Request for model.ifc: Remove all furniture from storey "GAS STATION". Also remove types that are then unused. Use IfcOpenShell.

First a look at what the model holds.

```python
import ifcopenshell
import ifcopenshell.util.element

model = ifcopenshell.open("model.ifc")
print(model.schema)
storey = next(s for s in model.by_type("IfcBuildingStorey") if s.Name == "GAS STATION")
furniture = [e for e in ifcopenshell.util.element.get_decomposition(storey) if e.is_a("IfcFurnishingElement")]
seen = {}
for e in furniture:
    element_type = ifcopenshell.util.element.get_type(e)
    name = element_type.Name if element_type not in (None, e) else None
    seen[name] = seen.get(name, 0) + 1
for name, count in sorted(seen.items(), key=str):
    print(count, "x", name)
```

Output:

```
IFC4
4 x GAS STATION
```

```python
import ifcopenshell
import ifcopenshell.api.root
import ifcopenshell.util.element

model = ifcopenshell.open("model.ifc")

storey = next(s for s in model.by_type("IfcBuildingStorey") if s.Name == "GAS STATION")
furniture = [e for e in ifcopenshell.util.element.get_decomposition(storey) if e.is_a("IfcFurnishingElement")]
types = {ifcopenshell.util.element.get_type(e) for e in furniture} - {None, *furniture}

for e in furniture:
    ifcopenshell.api.root.remove_product(model, product=e)
print(len(furniture), "removed")

unused = [t for t in types if not ifcopenshell.util.element.get_types(t)]
for t in unused:
    ifcopenshell.api.root.remove_product(model, product=t)
print(len(unused), "unused types removed")

model.write("model_rev.ifc")
```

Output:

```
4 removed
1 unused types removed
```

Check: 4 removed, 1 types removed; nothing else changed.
